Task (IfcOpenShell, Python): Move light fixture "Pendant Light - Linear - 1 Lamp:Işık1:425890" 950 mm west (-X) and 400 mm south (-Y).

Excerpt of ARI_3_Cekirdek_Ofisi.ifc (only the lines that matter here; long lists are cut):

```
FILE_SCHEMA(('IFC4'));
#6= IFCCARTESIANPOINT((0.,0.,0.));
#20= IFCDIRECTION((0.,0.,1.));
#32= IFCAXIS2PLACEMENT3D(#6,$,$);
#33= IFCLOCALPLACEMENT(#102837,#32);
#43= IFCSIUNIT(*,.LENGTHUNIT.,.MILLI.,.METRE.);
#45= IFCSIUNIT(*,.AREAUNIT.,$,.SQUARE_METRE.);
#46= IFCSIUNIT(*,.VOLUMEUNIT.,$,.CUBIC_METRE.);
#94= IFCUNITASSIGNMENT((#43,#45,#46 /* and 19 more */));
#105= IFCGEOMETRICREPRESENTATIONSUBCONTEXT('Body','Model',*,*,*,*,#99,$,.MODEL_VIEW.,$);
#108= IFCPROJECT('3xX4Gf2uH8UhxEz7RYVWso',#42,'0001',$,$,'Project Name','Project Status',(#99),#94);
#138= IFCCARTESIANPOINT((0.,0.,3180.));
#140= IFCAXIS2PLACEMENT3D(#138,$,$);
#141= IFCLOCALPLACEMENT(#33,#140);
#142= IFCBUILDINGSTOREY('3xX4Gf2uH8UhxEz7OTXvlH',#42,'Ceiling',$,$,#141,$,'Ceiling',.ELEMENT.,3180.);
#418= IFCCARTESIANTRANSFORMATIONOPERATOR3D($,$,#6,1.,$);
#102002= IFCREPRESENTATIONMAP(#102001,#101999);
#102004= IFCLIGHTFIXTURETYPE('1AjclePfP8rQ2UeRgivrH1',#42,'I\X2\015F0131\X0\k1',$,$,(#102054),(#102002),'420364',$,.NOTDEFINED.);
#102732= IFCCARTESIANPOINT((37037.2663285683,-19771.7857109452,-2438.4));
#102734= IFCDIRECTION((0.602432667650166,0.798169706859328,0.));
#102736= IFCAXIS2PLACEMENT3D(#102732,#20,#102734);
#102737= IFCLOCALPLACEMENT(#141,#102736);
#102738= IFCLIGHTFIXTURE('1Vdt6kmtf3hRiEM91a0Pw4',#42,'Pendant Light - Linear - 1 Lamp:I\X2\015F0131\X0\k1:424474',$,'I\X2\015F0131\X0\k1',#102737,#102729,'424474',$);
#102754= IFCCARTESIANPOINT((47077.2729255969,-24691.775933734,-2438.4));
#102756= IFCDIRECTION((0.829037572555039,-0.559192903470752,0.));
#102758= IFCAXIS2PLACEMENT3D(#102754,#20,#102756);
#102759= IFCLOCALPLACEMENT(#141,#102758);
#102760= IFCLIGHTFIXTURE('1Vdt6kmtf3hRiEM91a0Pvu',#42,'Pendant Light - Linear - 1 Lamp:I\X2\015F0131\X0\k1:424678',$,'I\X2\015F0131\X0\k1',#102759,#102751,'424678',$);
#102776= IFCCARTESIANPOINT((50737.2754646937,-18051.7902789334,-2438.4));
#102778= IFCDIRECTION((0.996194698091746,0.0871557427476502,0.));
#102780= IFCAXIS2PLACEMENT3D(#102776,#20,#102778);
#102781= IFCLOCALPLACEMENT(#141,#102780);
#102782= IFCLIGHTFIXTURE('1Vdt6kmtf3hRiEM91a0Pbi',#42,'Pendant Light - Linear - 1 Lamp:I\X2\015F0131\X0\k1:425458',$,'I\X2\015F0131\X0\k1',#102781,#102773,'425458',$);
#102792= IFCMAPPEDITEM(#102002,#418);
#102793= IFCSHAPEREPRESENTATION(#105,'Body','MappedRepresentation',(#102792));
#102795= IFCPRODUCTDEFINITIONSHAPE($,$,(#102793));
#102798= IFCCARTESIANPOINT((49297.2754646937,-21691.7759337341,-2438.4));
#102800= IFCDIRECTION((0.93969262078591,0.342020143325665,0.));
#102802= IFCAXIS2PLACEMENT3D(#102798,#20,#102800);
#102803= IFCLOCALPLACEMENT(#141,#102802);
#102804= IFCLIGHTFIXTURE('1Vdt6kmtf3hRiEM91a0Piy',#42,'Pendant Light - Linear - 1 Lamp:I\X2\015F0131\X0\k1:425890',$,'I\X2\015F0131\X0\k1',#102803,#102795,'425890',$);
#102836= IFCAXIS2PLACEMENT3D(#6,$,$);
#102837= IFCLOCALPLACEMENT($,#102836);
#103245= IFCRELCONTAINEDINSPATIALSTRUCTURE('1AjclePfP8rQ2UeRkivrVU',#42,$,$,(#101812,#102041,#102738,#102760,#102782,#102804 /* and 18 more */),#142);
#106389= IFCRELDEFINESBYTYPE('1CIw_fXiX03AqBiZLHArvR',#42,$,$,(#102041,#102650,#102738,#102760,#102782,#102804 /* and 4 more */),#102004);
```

```python
import ifcopenshell
import ifcopenshell.api.geometry
import ifcopenshell.util.placement
import ifcopenshell.util.unit

model = ifcopenshell.open("ARI_3_Cekirdek_Ofisi.ifc")
unit_scale = ifcopenshell.util.unit.calculate_unit_scale(model)

item = model.by_id(102804)
matrix = ifcopenshell.util.placement.get_local_placement(item.ObjectPlacement)
matrix[0, 3] -= 0.95 / unit_scale
matrix[1, 3] -= 0.4 / unit_scale
ifcopenshell.api.geometry.edit_object_placement(model, product=item, matrix=matrix, is_si=False)

print(ifcopenshell.util.placement.get_local_placement(item.ObjectPlacement).round(3) + 0.0)

model.write("ARI_3_Cekirdek_Ofisi_edited.ifc")
```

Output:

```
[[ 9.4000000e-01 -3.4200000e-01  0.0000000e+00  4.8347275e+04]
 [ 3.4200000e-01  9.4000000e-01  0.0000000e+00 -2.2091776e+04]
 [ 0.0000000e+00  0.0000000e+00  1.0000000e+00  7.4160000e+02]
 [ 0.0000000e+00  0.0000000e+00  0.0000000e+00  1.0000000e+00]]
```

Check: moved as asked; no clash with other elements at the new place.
